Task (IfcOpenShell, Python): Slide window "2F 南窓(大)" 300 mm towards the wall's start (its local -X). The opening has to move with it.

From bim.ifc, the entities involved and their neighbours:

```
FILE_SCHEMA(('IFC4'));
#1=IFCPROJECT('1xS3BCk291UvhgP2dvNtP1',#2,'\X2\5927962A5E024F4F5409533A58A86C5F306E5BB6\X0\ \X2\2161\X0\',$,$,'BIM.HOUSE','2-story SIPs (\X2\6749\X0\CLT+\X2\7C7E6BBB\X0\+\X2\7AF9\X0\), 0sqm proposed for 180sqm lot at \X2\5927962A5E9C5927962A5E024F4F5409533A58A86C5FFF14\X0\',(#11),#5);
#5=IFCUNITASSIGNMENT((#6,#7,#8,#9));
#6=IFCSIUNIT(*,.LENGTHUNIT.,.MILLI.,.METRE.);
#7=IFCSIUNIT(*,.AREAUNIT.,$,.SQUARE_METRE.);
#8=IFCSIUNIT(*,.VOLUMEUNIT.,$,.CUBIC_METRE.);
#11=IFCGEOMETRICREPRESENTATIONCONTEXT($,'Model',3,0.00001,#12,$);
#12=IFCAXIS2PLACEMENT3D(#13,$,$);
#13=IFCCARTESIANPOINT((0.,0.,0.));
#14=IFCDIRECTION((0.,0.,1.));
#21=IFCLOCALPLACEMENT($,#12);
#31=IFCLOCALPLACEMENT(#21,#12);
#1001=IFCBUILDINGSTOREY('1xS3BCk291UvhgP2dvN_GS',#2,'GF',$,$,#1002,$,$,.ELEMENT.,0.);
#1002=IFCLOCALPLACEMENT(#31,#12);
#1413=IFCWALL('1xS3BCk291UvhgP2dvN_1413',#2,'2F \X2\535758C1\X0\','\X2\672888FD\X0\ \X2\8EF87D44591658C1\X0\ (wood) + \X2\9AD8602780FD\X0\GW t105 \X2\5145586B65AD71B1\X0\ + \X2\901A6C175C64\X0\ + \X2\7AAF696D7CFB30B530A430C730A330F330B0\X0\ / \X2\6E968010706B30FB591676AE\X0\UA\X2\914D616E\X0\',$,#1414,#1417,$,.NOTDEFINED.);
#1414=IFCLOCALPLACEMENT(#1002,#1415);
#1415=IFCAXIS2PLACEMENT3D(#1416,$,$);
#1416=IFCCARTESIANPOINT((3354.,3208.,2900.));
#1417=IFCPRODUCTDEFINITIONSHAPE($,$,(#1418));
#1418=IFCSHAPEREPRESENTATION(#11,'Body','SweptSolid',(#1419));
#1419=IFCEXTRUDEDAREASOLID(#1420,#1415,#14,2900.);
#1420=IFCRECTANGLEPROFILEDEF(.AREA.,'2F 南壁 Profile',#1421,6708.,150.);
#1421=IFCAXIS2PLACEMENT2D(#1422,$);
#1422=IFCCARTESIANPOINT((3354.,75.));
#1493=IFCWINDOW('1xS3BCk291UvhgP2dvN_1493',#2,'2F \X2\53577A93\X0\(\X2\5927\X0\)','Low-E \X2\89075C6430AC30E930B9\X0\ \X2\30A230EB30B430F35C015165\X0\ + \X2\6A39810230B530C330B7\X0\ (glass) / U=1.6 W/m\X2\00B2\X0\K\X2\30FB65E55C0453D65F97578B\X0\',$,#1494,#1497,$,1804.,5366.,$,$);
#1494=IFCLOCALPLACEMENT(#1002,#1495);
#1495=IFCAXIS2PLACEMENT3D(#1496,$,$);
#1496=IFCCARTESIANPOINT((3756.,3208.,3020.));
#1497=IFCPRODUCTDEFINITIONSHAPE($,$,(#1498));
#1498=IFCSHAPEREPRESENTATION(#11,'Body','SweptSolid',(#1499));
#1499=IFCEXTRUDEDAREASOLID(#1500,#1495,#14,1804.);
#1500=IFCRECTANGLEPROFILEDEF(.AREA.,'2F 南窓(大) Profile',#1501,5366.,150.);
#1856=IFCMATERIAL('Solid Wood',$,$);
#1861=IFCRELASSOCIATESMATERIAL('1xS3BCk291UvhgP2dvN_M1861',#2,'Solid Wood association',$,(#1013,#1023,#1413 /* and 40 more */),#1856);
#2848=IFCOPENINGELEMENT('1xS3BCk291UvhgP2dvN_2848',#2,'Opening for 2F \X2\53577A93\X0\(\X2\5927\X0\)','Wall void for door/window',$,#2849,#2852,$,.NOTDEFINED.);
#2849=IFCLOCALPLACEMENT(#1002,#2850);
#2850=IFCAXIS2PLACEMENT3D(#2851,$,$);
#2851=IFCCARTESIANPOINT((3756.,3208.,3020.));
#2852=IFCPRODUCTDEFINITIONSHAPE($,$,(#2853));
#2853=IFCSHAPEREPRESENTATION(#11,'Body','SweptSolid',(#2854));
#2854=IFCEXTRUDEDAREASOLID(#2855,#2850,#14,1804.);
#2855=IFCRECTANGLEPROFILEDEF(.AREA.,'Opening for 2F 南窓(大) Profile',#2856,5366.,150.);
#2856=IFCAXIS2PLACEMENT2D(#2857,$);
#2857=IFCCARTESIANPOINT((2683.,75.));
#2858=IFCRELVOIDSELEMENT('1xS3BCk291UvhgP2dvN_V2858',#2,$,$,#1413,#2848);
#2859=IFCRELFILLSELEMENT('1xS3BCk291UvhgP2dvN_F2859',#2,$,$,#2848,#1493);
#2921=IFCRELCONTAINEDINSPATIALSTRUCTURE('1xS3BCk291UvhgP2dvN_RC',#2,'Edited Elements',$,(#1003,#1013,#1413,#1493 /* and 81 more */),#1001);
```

```python
import ifcopenshell
import ifcopenshell.api.geometry
import ifcopenshell.util.placement
import ifcopenshell.util.unit

model = ifcopenshell.open("bim.ifc")
unit_scale = ifcopenshell.util.unit.calculate_unit_scale(model)

window = model.by_guid("1xS3BCk291UvhgP2dvN_1493")
opening = window.FillsVoids[0].RelatingOpeningElement
wall = opening.VoidsElements[0].RelatingBuildingElement

wall_matrix = ifcopenshell.util.placement.get_local_placement(wall.ObjectPlacement)
shift = wall_matrix[:3, 0] * -0.3 / unit_scale
before = ifcopenshell.util.placement.get_local_placement(window.ObjectPlacement)[:3, 3].copy()

# The window is not placed relative to its opening, so move both.
for product in (opening, window):
    matrix = ifcopenshell.util.placement.get_local_placement(product.ObjectPlacement)
    matrix[:3, 3] += shift
    ifcopenshell.api.geometry.edit_object_placement(model, product=product, matrix=matrix, is_si=False)

after = ifcopenshell.util.placement.get_local_placement(window.ObjectPlacement)[:3, 3]
print("window moved by", (after - before).round(3) + 0.0)

model.write("bim_rev.ifc")
```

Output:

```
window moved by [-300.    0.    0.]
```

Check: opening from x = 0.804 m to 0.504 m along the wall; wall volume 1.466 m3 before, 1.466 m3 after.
